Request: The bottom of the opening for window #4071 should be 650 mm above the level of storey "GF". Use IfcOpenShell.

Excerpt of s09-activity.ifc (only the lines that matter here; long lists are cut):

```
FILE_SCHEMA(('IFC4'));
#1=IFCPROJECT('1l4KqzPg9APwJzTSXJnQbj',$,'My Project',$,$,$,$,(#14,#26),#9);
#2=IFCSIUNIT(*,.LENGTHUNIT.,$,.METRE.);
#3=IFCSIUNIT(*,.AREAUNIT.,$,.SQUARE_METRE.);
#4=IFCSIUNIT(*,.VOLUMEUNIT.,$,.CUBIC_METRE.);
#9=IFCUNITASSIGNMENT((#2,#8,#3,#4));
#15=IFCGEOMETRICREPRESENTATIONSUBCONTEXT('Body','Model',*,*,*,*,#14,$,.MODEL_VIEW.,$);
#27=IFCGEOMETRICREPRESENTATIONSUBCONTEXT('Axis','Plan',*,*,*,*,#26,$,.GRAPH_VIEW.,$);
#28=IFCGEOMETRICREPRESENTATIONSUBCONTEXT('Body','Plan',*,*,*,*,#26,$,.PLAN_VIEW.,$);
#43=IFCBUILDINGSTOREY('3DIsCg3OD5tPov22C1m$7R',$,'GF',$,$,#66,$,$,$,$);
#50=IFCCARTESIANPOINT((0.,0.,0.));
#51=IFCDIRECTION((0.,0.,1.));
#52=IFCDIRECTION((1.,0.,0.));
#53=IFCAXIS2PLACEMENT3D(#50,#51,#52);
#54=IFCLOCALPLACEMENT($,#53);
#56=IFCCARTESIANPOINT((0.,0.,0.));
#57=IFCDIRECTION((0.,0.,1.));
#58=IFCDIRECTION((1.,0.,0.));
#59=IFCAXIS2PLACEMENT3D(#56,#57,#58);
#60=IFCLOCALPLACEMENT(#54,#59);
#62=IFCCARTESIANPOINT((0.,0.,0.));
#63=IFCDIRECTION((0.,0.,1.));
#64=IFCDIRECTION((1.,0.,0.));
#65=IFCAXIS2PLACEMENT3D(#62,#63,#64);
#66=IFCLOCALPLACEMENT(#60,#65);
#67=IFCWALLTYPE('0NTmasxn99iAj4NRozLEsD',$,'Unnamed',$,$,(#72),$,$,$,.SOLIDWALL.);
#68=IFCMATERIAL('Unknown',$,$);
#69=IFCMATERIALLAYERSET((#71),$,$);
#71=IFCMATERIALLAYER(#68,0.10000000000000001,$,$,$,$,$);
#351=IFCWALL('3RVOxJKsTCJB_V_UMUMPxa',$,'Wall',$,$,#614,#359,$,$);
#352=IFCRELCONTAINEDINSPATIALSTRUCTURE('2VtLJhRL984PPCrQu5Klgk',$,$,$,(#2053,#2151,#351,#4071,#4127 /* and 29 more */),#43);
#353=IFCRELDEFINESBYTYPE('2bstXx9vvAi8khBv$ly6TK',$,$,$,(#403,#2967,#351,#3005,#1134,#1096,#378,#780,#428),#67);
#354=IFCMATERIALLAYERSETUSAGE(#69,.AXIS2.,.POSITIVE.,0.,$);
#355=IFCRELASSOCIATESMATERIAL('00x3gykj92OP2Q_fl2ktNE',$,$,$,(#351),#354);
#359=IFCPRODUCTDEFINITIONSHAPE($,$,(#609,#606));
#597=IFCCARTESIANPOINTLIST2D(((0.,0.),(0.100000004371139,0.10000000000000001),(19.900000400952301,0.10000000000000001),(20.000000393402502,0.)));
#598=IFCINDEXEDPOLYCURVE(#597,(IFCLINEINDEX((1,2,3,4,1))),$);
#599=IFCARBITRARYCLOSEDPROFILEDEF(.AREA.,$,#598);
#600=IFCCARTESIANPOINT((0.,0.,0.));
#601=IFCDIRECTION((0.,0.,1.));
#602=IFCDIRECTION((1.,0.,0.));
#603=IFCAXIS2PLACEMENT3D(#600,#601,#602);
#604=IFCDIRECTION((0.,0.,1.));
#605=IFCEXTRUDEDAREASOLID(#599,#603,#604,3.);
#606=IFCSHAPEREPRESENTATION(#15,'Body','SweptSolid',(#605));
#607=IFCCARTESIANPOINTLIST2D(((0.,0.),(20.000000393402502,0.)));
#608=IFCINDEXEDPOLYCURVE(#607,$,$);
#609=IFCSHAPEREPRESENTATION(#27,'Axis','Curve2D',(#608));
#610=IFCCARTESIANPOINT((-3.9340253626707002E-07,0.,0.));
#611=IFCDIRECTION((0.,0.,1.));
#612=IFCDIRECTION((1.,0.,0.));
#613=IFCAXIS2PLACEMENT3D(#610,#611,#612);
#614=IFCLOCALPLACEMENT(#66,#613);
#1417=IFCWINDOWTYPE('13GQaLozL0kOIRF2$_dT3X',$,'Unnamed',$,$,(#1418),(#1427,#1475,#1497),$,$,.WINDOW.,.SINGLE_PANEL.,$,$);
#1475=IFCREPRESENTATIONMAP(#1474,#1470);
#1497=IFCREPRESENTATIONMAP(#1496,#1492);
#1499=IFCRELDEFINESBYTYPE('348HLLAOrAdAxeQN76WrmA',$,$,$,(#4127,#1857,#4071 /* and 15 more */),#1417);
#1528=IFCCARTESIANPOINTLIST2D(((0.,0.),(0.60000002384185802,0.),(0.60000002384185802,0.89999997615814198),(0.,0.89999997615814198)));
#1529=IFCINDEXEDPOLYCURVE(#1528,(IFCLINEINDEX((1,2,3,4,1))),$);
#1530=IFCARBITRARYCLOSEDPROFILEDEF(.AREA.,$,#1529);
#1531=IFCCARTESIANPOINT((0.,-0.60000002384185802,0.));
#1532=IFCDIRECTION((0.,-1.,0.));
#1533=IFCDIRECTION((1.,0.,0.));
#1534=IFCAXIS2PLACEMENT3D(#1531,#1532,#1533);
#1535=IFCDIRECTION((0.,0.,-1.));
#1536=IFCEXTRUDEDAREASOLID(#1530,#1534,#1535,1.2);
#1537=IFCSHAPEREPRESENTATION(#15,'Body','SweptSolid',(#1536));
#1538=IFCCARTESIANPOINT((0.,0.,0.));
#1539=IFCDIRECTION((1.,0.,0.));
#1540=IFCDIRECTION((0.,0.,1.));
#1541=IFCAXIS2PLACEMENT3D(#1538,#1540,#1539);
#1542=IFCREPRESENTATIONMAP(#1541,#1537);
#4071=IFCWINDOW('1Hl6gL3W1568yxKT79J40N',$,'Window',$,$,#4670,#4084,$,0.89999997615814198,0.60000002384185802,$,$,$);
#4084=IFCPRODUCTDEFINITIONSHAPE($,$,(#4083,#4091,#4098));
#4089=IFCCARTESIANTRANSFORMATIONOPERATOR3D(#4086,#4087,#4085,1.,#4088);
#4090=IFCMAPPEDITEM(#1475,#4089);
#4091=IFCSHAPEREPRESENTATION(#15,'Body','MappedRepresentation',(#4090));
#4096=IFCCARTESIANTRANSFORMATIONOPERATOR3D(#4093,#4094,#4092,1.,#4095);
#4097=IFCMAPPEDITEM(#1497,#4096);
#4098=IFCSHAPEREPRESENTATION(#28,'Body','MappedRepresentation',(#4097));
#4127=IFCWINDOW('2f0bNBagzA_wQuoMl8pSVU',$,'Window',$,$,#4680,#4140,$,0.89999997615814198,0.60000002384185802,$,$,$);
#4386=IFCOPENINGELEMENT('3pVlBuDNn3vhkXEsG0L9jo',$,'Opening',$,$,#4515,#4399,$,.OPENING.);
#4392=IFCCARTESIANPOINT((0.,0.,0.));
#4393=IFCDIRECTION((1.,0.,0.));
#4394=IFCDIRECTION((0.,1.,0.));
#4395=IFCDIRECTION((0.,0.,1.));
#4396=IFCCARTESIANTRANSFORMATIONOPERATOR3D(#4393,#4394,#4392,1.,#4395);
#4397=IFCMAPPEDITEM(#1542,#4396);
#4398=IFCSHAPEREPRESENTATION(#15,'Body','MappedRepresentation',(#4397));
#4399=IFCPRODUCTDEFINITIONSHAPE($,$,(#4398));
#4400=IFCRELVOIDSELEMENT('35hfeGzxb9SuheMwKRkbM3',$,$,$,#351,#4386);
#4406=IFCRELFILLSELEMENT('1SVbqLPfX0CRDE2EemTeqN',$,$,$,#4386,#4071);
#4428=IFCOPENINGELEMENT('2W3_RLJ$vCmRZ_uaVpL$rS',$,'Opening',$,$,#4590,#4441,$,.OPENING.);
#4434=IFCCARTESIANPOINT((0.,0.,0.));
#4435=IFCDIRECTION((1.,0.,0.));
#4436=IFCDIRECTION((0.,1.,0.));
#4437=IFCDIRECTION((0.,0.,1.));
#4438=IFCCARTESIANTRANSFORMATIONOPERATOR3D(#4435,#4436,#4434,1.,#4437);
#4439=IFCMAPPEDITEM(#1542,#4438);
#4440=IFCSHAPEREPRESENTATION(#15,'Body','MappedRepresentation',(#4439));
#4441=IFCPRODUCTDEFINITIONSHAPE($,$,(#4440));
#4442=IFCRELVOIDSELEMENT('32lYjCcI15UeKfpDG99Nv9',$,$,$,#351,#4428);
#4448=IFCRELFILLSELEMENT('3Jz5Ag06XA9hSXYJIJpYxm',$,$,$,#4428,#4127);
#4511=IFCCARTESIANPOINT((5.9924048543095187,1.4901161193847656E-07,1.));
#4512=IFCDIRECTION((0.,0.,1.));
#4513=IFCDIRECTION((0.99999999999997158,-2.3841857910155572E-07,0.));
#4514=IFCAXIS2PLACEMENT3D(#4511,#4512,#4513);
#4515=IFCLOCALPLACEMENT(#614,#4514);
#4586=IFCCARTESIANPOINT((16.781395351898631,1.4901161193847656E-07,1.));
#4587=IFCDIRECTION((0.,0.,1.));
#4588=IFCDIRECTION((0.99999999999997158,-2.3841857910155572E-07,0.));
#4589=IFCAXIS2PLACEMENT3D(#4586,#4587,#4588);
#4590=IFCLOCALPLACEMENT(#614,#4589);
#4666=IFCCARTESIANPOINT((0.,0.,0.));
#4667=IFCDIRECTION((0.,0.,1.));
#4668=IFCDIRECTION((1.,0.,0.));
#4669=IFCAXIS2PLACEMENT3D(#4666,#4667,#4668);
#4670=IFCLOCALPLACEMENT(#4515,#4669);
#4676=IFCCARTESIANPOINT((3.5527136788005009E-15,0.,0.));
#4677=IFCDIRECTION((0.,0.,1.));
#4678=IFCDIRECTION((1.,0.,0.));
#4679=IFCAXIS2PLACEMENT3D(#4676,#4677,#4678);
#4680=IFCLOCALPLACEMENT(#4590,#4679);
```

```python
import numpy as np
import ifcopenshell
import ifcopenshell.api.geometry
import ifcopenshell.geom
import ifcopenshell.util.element
import ifcopenshell.util.placement
import ifcopenshell.util.shape
import ifcopenshell.util.unit

model = ifcopenshell.open("s09-activity.ifc")
unit_scale = ifcopenshell.util.unit.calculate_unit_scale(model)

window = model.by_guid("1Hl6gL3W1568yxKT79J40N")
opening = window.FillsVoids[0].RelatingOpeningElement
storey = ifcopenshell.util.element.get_container(window, ifc_class="IfcBuildingStorey")
level = ifcopenshell.util.placement.get_local_placement(storey.ObjectPlacement)[2, 3]

# The opening's origin need not be at the sill, so measure its lowest point.
shape = ifcopenshell.geom.create_shape(ifcopenshell.geom.settings(), opening)
bottom = ifcopenshell.util.shape.get_shape_bottom_elevation(shape, shape.geometry) / unit_scale
dz = level + 0.65 / unit_scale - bottom

shift = np.array([0.0, 0.0, dz])
# The window is placed relative to its opening, so it follows when the opening moves.
matrix = ifcopenshell.util.placement.get_local_placement(opening.ObjectPlacement)
matrix[:3, 3] += shift
ifcopenshell.api.geometry.edit_object_placement(
    model, product=opening, matrix=matrix, is_si=False, should_transform_children=True
)

print(f"moved by {dz * unit_scale:+.3f} m")

model.write("s09-activity_updated.ifc")
```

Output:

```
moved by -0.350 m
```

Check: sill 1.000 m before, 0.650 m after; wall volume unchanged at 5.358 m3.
